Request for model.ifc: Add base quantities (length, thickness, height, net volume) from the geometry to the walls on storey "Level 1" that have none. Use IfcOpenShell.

First a look at what the model holds.

```python
import ifcopenshell
import ifcopenshell.util.element
import ifcopenshell.util.unit

model = ifcopenshell.open("model.ifc")
print(model.schema)
for unit_type in ("LENGTHUNIT", "AREAUNIT", "VOLUMEUNIT"):
    print(unit_type, ifcopenshell.util.unit.calculate_unit_scale(model, unit_type))
storey = next(s for s in model.by_type("IfcBuildingStorey") if s.Name == "Level 1")
walls = [e for e in ifcopenshell.util.element.get_decomposition(storey) if e.is_a("IfcWall")]
for e in sorted(walls, key=lambda e: e.id()):
    print(e.id(), e.is_a(), e.Name, list(ifcopenshell.util.element.get_psets(e, qtos_only=True)), sep=" | ")
```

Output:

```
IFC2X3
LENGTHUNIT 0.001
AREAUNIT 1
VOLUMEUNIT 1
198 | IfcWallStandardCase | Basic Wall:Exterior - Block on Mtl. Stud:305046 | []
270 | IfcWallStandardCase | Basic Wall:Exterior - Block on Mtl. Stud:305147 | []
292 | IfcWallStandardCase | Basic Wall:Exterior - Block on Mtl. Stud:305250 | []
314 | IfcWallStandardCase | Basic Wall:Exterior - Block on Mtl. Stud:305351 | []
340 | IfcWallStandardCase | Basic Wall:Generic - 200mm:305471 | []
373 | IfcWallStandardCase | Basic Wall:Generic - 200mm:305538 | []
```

```python
import ifcopenshell
import ifcopenshell.api.pset
import ifcopenshell.geom
import ifcopenshell.util.element
import ifcopenshell.util.shape
import ifcopenshell.util.unit

model = ifcopenshell.open("model.ifc")
unit_scale = ifcopenshell.util.unit.calculate_unit_scale(model)
volume_scale = ifcopenshell.util.unit.calculate_unit_scale(model, "VOLUMEUNIT")
settings = ifcopenshell.geom.settings()

storey = next(s for s in model.by_type("IfcBuildingStorey") if s.Name == "Level 1")
walls = [e for e in ifcopenshell.util.element.get_decomposition(storey) if e.is_a("IfcWall")]

for e in sorted(walls, key=lambda e: e.id()):
    if ifcopenshell.util.element.get_psets(e, qtos_only=True, should_inherit=False):
        continue
    # Geometry comes back in metres, in the element's own axes.
    shape = ifcopenshell.geom.create_shape(settings, e)
    values = {
        "Length": ifcopenshell.util.shape.get_x(shape.geometry) / unit_scale,
        "Width": ifcopenshell.util.shape.get_y(shape.geometry) / unit_scale,
        "Height": ifcopenshell.util.shape.get_z(shape.geometry) / unit_scale,
        "NetVolume": ifcopenshell.util.shape.get_volume(shape.geometry) / volume_scale,
    }
    qto = ifcopenshell.api.pset.add_qto(model, product=e, name="BaseQuantities")
    ifcopenshell.api.pset.edit_qto(model, qto=qto, properties=values)
    print(e.id(), {k: round(v, 3) for k, v in values.items()})

model.write("model_updated.ifc")
```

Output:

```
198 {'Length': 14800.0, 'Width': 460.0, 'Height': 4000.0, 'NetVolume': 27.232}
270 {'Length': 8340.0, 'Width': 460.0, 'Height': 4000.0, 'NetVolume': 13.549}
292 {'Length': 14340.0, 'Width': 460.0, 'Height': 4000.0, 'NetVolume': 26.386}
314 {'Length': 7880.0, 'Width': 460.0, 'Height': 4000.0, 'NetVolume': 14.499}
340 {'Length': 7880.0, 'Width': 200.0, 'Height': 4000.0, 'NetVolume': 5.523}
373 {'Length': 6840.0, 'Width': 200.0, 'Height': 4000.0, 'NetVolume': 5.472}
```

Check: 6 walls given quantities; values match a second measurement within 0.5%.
